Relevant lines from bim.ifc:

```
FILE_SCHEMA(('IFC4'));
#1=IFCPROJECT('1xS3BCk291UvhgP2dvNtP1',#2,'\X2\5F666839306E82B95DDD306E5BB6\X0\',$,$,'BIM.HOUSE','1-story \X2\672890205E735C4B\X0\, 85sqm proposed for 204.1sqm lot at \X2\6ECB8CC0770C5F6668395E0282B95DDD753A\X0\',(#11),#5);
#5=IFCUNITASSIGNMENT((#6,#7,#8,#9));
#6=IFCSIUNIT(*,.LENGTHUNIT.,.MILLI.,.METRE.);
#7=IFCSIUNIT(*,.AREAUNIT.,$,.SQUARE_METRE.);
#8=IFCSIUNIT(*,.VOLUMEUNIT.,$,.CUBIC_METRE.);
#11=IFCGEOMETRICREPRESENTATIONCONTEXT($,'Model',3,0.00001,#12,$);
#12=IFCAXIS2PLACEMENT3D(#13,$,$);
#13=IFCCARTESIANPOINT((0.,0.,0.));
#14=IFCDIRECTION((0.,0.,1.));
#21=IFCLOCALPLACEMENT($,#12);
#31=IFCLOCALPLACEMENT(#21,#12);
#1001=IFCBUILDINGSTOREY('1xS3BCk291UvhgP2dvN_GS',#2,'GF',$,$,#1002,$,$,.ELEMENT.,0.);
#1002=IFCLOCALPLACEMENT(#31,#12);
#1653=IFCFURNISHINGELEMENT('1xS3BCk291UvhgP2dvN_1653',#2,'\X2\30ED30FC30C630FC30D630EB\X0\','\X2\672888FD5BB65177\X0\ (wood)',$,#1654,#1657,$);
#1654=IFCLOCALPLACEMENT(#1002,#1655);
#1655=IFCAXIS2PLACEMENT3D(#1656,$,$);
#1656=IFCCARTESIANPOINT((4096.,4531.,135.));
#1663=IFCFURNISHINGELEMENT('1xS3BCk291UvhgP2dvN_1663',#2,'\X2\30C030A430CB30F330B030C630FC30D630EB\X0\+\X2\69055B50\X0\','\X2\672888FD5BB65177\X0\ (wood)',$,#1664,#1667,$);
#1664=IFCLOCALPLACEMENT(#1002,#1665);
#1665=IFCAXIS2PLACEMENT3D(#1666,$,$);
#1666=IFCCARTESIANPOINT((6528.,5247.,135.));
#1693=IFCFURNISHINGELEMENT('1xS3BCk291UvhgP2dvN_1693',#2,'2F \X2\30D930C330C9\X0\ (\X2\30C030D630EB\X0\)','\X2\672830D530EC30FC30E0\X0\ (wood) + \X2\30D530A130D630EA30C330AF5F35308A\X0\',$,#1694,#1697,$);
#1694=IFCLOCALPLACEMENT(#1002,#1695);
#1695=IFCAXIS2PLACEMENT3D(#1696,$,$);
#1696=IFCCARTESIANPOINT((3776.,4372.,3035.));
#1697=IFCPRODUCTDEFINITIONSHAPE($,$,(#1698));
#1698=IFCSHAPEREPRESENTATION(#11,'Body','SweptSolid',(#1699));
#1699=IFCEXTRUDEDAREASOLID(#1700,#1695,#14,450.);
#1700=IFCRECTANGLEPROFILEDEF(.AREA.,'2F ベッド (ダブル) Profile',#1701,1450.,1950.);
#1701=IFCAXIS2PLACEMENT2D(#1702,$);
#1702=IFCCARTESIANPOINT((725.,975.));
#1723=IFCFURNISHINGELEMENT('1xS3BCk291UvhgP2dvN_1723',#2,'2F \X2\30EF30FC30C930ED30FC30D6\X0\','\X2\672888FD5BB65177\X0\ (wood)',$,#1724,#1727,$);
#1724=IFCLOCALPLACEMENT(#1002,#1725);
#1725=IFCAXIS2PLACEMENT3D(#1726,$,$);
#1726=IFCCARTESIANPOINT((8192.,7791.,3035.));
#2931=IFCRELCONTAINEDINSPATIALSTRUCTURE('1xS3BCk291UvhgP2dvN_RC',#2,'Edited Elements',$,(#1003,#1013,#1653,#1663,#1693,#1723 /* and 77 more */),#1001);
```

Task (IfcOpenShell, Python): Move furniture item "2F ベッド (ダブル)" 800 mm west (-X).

```python
import ifcopenshell
import ifcopenshell.api.geometry
import ifcopenshell.util.placement

model = ifcopenshell.open("bim.ifc")

item = model.by_guid("1xS3BCk291UvhgP2dvN_1693")
matrix = ifcopenshell.util.placement.get_local_placement(item.ObjectPlacement)
matrix[0, 3] -= 800.0
ifcopenshell.api.geometry.edit_object_placement(model, product=item, matrix=matrix, is_si=False)

print(ifcopenshell.util.placement.get_local_placement(item.ObjectPlacement).round(3) + 0.0)

model.write("bim-out.ifc")
```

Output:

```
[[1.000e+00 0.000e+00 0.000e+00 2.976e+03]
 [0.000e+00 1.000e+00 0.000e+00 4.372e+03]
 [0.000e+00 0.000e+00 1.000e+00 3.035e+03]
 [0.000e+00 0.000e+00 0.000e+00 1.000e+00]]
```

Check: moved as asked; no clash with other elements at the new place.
